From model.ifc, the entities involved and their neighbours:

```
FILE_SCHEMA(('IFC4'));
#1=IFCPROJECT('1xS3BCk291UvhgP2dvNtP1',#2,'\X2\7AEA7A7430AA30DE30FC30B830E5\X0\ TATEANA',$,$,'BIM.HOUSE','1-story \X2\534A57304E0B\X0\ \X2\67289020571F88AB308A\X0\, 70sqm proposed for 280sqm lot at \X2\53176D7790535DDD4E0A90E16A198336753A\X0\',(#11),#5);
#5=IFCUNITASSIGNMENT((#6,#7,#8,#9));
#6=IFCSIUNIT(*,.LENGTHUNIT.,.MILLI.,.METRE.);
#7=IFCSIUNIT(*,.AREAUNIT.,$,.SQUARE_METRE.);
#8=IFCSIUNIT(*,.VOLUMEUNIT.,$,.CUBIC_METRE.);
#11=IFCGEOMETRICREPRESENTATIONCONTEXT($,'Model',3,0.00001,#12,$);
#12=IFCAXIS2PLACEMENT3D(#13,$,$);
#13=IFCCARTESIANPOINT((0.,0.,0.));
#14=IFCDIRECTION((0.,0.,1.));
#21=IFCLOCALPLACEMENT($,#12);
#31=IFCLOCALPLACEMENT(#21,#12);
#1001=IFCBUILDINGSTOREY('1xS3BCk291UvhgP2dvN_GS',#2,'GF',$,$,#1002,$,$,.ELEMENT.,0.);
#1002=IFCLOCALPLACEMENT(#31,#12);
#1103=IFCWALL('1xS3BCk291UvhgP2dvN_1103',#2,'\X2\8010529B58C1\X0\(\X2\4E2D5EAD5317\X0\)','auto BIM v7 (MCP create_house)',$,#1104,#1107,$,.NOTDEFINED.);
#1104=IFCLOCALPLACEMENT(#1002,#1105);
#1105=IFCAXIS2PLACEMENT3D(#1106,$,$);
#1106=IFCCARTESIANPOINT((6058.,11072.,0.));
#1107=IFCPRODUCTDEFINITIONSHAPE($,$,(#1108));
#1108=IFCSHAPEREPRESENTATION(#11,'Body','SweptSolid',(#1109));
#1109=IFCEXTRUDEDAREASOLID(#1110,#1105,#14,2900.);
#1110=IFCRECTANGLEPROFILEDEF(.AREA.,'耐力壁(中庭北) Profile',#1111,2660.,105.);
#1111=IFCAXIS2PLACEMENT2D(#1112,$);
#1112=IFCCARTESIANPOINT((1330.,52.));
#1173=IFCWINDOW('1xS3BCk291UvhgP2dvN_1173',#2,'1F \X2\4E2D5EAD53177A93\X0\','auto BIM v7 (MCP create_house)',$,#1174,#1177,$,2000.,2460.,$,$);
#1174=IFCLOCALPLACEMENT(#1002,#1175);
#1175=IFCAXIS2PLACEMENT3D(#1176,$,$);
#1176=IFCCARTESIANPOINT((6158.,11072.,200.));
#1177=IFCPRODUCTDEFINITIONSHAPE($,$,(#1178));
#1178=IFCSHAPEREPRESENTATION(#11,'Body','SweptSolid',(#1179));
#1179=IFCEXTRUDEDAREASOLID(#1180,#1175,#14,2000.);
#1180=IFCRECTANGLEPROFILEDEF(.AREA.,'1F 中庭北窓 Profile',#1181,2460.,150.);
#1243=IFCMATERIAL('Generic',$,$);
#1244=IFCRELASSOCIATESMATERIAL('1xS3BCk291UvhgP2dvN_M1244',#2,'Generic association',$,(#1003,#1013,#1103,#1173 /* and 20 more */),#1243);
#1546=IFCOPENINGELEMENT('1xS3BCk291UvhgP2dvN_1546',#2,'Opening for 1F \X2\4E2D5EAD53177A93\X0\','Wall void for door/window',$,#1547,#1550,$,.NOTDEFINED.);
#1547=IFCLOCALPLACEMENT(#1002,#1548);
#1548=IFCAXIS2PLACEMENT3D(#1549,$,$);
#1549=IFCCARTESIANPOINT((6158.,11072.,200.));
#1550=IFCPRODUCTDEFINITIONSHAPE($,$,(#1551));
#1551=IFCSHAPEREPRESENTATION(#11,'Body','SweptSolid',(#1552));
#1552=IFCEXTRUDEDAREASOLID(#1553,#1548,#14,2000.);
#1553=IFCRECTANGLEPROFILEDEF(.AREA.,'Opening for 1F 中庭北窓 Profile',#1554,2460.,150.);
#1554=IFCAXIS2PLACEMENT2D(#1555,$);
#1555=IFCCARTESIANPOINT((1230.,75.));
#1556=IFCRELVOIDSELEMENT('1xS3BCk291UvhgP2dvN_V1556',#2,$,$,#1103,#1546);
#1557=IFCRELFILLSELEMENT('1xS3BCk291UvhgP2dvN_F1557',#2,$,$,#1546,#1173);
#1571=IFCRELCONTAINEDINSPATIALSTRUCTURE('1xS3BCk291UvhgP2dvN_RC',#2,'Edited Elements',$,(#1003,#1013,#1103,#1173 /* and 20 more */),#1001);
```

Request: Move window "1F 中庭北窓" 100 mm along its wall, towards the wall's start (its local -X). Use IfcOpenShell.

```python
import ifcopenshell
import ifcopenshell.api.geometry
import ifcopenshell.util.placement
import ifcopenshell.util.unit

model = ifcopenshell.open("model.ifc")
unit_scale = ifcopenshell.util.unit.calculate_unit_scale(model)

window = model.by_guid("1xS3BCk291UvhgP2dvN_1173")
opening = window.FillsVoids[0].RelatingOpeningElement
wall = opening.VoidsElements[0].RelatingBuildingElement

wall_matrix = ifcopenshell.util.placement.get_local_placement(wall.ObjectPlacement)
shift = wall_matrix[:3, 0] * -0.1 / unit_scale
before = ifcopenshell.util.placement.get_local_placement(window.ObjectPlacement)[:3, 3].copy()

# The window is not placed relative to its opening, so move both.
for product in (opening, window):
    matrix = ifcopenshell.util.placement.get_local_placement(product.ObjectPlacement)
    matrix[:3, 3] += shift
    ifcopenshell.api.geometry.edit_object_placement(model, product=product, matrix=matrix, is_si=False)

after = ifcopenshell.util.placement.get_local_placement(window.ObjectPlacement)[:3, 3]
print("window moved by", (after - before).round(3) + 0.0)

model.write("model_rev.ifc")
```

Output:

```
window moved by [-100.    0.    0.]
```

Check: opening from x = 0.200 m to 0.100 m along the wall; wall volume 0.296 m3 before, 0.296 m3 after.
